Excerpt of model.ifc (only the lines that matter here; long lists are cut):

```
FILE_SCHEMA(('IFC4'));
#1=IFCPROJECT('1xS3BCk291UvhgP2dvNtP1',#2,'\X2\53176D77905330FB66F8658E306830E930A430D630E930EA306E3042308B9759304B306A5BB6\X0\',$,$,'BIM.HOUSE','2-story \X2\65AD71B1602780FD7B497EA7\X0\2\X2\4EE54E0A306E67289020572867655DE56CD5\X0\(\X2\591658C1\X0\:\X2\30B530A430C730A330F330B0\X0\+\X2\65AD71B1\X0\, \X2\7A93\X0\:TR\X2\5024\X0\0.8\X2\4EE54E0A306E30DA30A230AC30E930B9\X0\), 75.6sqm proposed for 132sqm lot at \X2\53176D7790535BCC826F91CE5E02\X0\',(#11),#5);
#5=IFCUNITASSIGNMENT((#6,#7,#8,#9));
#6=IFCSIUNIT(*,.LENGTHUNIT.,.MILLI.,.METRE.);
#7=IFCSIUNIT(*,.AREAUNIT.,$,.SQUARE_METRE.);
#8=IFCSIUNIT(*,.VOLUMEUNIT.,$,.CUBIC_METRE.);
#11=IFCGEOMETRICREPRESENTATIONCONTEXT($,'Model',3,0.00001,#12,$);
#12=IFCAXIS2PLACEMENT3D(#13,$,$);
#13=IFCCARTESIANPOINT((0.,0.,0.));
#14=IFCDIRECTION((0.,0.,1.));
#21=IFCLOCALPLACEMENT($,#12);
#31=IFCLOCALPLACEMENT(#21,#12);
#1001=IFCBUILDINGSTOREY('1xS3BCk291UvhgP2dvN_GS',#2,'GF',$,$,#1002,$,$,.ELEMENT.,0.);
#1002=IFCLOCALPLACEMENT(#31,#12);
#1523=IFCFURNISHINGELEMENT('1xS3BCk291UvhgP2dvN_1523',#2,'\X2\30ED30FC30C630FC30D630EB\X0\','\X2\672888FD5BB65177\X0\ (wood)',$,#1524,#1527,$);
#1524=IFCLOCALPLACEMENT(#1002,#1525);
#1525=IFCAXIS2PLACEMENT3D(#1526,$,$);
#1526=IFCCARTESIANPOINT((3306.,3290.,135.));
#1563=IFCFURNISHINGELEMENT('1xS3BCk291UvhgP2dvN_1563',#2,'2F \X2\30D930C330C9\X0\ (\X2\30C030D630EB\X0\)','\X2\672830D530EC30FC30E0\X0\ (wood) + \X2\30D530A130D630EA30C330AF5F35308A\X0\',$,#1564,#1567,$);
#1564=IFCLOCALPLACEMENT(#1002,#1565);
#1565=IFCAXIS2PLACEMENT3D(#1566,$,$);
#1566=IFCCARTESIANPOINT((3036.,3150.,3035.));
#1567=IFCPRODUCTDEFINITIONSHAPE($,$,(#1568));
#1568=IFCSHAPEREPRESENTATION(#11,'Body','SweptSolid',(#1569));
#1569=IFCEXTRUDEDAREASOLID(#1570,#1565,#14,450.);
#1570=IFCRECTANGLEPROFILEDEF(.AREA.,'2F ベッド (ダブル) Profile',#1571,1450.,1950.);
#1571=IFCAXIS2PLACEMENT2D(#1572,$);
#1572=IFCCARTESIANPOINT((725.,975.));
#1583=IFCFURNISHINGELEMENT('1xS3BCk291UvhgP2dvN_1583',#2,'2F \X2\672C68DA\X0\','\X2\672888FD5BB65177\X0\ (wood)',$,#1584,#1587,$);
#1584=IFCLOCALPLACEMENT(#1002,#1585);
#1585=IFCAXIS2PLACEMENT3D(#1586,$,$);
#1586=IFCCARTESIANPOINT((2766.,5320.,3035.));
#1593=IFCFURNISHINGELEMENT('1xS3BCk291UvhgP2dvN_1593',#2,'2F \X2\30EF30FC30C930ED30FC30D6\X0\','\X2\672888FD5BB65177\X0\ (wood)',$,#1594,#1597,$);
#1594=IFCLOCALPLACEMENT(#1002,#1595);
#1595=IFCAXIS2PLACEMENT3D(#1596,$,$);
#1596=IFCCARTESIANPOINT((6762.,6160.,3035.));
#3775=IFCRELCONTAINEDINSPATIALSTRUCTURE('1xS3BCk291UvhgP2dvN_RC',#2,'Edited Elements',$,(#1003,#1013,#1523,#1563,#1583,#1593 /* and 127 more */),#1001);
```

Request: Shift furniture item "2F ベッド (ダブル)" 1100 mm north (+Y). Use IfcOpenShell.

```python
import ifcopenshell
import ifcopenshell.api.geometry
import ifcopenshell.util.placement
import ifcopenshell.util.unit

model = ifcopenshell.open("model.ifc")
unit_scale = ifcopenshell.util.unit.calculate_unit_scale(model)

item = model.by_id(1563)
matrix = ifcopenshell.util.placement.get_local_placement(item.ObjectPlacement)
matrix[1, 3] += 1.1 / unit_scale
ifcopenshell.api.geometry.edit_object_placement(model, product=item, matrix=matrix, is_si=False)

print(ifcopenshell.util.placement.get_local_placement(item.ObjectPlacement).round(3) + 0.0)

model.write("model_updated.ifc")
```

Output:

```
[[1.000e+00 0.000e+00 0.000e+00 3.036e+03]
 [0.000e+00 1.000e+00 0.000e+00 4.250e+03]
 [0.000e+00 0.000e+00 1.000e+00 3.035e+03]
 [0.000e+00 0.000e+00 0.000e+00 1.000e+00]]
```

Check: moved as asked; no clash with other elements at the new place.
